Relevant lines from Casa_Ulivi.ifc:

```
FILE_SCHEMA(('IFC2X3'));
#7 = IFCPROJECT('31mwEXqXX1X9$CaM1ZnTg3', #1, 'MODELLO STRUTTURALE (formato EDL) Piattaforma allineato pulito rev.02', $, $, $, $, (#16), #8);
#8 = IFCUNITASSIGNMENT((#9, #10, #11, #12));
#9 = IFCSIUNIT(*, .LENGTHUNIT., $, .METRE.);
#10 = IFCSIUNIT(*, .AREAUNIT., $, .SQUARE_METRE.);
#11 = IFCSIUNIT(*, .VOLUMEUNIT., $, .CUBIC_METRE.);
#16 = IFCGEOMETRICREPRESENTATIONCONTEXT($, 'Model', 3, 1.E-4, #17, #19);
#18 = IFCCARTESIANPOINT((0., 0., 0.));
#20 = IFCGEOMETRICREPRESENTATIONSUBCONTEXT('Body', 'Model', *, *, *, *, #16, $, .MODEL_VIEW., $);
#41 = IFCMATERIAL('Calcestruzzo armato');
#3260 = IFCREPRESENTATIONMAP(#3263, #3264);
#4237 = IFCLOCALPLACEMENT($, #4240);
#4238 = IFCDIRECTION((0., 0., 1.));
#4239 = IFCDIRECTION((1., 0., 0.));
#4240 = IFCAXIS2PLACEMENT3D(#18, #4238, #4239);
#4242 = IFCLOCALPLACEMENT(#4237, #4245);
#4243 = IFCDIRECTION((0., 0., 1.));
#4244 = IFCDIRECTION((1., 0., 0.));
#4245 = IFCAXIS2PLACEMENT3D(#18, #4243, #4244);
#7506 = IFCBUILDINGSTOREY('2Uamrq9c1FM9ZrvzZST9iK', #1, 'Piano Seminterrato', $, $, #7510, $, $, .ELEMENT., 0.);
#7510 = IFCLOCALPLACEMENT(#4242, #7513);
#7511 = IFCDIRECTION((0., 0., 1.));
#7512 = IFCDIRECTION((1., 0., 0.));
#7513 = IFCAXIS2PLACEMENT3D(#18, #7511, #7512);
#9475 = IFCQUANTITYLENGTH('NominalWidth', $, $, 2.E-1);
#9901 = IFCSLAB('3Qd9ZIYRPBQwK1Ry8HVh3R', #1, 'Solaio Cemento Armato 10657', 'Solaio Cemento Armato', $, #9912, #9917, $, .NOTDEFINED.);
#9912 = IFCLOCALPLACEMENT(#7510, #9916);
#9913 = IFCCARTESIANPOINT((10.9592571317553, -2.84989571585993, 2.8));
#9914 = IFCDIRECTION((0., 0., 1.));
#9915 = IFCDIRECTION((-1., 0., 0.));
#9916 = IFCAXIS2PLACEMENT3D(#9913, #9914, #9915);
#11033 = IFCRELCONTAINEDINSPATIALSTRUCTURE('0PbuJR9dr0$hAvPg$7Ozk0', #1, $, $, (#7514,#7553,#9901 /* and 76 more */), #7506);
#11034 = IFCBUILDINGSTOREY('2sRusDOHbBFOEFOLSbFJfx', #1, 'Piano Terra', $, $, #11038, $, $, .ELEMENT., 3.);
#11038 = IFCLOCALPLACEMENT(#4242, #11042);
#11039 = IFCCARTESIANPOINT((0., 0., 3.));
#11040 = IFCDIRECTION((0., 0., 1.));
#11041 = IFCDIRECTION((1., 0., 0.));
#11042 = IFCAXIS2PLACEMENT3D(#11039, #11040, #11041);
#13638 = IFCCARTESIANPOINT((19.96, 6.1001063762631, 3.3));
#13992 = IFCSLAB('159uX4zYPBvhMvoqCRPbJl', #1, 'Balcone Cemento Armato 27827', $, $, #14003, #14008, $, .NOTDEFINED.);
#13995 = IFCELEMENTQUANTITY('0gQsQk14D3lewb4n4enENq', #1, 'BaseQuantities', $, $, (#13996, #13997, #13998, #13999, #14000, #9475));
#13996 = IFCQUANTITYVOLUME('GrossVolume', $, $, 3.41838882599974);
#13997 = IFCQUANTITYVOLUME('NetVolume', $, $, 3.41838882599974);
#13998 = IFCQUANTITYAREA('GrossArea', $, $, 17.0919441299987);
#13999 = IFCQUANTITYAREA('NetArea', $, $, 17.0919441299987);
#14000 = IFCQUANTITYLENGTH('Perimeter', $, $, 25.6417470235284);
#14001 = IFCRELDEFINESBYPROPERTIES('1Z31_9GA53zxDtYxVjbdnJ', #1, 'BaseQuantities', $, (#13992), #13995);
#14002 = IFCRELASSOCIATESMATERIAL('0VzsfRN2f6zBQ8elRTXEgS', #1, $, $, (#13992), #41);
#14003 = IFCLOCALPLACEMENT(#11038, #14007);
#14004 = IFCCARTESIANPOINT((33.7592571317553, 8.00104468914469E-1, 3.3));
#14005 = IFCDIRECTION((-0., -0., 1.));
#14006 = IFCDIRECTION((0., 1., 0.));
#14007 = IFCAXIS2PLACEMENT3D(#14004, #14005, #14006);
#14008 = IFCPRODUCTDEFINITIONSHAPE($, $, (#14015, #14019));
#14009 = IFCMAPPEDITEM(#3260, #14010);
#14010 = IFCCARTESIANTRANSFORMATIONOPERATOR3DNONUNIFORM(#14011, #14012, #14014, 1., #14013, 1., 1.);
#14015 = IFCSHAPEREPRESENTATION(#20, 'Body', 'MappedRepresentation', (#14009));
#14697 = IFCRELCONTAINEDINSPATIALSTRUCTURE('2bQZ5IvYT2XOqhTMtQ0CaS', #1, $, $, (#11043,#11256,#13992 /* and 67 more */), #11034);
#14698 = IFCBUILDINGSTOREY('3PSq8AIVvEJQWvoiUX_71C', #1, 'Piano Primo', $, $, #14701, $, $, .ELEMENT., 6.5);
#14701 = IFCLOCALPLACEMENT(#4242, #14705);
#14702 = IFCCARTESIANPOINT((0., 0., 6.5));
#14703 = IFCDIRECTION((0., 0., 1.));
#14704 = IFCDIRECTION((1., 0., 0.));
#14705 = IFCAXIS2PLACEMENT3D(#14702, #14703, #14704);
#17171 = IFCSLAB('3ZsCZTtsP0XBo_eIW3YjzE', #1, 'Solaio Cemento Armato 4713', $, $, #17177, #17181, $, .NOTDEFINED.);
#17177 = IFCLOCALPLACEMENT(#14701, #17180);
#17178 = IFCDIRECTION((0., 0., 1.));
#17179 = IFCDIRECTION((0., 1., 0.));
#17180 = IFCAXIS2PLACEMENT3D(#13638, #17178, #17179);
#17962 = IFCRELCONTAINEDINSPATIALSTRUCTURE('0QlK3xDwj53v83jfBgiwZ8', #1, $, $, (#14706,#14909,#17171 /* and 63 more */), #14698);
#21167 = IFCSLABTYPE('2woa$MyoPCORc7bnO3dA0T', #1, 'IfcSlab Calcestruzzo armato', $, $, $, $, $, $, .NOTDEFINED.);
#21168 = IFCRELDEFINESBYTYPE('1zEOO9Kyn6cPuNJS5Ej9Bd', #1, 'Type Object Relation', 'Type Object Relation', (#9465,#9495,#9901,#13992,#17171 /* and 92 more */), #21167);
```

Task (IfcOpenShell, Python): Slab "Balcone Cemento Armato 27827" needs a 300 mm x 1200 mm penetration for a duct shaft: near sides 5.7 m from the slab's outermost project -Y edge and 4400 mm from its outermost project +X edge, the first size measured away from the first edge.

```python
import numpy as np
import ifcopenshell
import ifcopenshell.api.feature
import ifcopenshell.api.geometry
import ifcopenshell.api.pset
import ifcopenshell.api.root
import ifcopenshell.geom
import ifcopenshell.util.element
import ifcopenshell.util.placement
import ifcopenshell.util.representation
import ifcopenshell.util.shape
import ifcopenshell.util.unit

model = ifcopenshell.open("Casa_Ulivi.ifc")
unit_scale = ifcopenshell.util.unit.calculate_unit_scale(model)
area_scale = ifcopenshell.util.unit.calculate_unit_scale(model, "AREAUNIT")
volume_scale = ifcopenshell.util.unit.calculate_unit_scale(model, "VOLUMEUNIT")
settings = ifcopenshell.geom.settings()


def volume(element):
    """Net volume in cubic metres, openings subtracted."""
    shape = ifcopenshell.geom.create_shape(settings, element)
    return ifcopenshell.util.shape.get_volume(shape.geometry)


slab = model.by_id(13992)
before = volume(slab)

# Extent in the slab's own axes, in metres. The edges named are its -X and -Y sides.
slab_shape = ifcopenshell.geom.create_shape(settings, slab)
vertices = ifcopenshell.util.shape.get_vertices(slab_shape.geometry)
x_min, y_min, bottom = vertices.min(axis=0)
top = vertices[:, 2].max()

opening = ifcopenshell.api.root.create_entity(model, ifc_class="IfcOpeningElement", name="Duct shaft opening")
context = ifcopenshell.util.representation.get_context(model, "Model", "Body", "MODEL_VIEW")
width, depth = 0.3, 1.2
outline = [(0.0, 0.0), (width, 0.0), (width, depth), (0.0, depth), (0.0, 0.0)]
# Overshoot both faces by 50 mm so the cut is clean.
shape = ifcopenshell.api.geometry.add_slab_representation(
    model, context=context, depth=top - bottom + 0.1, polyline=outline
)
ifcopenshell.api.geometry.assign_representation(model, product=opening, representation=shape)

matrix = ifcopenshell.util.placement.get_local_placement(slab.ObjectPlacement)
matrix[:, 3] = matrix @ np.append(np.array([x_min + 5.7, y_min + 4.4, bottom - 0.05]) / unit_scale, 1.0)
ifcopenshell.api.geometry.edit_object_placement(model, product=opening, matrix=matrix, is_si=False)
ifcopenshell.api.feature.add_feature(model, feature=opening, element=slab)

after = volume(slab)

# Update the slab's stored quantities.
qto = model.by_id(ifcopenshell.util.element.get_pset(slab, "BaseQuantities", should_inherit=False)["id"])
ifcopenshell.api.pset.edit_qto(model, qto=qto, properties={
    "NetVolume": after / volume_scale,
    "NetArea": after / (top - bottom) / area_scale,
})

print(f"slab volume {before:.3f} -> {after:.3f} m3")

model.write("Casa_Ulivi_updated.ifc")
```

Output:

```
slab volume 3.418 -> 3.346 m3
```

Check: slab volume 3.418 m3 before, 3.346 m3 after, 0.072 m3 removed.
